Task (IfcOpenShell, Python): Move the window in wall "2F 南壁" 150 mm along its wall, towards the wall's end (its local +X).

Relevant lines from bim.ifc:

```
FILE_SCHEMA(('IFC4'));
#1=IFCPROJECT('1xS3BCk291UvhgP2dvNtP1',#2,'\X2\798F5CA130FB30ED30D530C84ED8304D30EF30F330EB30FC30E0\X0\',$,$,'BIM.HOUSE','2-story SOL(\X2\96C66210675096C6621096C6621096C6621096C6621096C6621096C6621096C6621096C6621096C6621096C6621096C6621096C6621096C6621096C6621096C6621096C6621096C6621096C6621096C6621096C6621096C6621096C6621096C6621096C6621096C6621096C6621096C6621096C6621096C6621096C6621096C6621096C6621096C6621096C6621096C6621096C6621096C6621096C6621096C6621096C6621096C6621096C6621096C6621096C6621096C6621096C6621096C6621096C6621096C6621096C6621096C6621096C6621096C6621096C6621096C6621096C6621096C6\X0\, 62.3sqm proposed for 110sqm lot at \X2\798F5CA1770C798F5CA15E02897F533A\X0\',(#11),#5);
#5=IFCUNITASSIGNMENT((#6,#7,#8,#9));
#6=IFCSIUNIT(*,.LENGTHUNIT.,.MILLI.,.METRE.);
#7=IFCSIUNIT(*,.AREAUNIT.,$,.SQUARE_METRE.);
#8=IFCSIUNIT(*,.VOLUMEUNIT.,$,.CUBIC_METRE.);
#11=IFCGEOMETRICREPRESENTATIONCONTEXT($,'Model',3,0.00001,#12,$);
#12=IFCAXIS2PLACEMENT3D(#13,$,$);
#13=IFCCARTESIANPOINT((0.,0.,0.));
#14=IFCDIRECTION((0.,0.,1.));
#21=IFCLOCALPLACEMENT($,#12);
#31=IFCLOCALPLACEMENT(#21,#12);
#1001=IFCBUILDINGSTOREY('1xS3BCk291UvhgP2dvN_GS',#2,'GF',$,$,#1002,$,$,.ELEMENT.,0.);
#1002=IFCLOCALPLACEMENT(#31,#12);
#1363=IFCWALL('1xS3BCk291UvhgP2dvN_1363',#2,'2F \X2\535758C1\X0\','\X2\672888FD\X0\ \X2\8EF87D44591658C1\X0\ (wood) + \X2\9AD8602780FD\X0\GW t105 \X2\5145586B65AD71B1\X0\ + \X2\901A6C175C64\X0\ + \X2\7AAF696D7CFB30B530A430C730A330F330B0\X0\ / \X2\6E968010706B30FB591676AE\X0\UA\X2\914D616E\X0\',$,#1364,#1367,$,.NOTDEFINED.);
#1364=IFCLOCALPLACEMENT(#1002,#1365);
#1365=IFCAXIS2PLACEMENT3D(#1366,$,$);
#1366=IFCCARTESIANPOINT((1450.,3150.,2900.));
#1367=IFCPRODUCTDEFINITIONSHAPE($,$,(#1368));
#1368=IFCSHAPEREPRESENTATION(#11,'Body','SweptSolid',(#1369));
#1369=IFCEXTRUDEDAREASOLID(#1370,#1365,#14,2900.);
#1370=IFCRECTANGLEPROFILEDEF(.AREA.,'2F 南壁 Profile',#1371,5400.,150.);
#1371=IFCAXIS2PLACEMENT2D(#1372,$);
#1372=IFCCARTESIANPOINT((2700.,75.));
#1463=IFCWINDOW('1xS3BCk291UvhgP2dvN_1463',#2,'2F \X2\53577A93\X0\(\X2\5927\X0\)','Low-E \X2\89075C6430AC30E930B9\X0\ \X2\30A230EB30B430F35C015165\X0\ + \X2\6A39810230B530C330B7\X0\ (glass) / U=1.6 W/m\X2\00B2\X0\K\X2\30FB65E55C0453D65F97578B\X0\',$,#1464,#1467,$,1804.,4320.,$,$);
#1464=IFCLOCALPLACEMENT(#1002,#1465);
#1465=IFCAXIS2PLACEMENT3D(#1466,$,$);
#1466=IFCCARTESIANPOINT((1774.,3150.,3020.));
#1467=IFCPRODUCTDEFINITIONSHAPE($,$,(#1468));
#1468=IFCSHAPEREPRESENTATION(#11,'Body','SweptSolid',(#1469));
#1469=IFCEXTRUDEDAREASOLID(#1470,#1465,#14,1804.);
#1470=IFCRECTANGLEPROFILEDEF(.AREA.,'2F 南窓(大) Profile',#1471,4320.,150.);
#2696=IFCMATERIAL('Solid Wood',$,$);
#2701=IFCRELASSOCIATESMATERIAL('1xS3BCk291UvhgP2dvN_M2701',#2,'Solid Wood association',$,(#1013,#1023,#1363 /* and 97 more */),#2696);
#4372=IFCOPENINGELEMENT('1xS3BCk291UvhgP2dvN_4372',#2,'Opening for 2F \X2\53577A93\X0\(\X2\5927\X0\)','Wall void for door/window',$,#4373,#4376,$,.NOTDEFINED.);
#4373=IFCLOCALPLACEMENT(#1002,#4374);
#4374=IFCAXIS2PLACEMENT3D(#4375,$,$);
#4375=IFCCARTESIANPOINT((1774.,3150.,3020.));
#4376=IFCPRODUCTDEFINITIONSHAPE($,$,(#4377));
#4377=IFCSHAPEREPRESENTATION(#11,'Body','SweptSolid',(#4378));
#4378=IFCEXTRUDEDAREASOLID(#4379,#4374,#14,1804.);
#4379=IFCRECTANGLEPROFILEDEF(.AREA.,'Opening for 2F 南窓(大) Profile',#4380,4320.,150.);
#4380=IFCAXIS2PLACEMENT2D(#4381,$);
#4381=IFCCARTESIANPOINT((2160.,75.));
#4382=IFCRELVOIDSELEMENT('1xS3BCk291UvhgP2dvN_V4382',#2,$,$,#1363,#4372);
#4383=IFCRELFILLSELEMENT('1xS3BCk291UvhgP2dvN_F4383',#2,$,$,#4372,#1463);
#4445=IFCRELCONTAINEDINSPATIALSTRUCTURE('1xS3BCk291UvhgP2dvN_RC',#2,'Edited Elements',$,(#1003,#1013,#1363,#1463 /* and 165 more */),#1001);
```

```python
import ifcopenshell
import ifcopenshell.api.geometry
import ifcopenshell.util.placement

model = ifcopenshell.open("bim.ifc")

window = model.by_id(1463)
opening = window.FillsVoids[0].RelatingOpeningElement
wall = opening.VoidsElements[0].RelatingBuildingElement

wall_matrix = ifcopenshell.util.placement.get_local_placement(wall.ObjectPlacement)
shift = wall_matrix[:3, 0] * 150.0
before = ifcopenshell.util.placement.get_local_placement(window.ObjectPlacement)[:3, 3].copy()

# The window is not placed relative to its opening, so move both.
for product in (opening, window):
    matrix = ifcopenshell.util.placement.get_local_placement(product.ObjectPlacement)
    matrix[:3, 3] += shift
    ifcopenshell.api.geometry.edit_object_placement(model, product=product, matrix=matrix, is_si=False)

after = ifcopenshell.util.placement.get_local_placement(window.ObjectPlacement)[:3, 3]
print("window moved by", (after - before).round(3) + 0.0)

model.write("bim_rev.ifc")
```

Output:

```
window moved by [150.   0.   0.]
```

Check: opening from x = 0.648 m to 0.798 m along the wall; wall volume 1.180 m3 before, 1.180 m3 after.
